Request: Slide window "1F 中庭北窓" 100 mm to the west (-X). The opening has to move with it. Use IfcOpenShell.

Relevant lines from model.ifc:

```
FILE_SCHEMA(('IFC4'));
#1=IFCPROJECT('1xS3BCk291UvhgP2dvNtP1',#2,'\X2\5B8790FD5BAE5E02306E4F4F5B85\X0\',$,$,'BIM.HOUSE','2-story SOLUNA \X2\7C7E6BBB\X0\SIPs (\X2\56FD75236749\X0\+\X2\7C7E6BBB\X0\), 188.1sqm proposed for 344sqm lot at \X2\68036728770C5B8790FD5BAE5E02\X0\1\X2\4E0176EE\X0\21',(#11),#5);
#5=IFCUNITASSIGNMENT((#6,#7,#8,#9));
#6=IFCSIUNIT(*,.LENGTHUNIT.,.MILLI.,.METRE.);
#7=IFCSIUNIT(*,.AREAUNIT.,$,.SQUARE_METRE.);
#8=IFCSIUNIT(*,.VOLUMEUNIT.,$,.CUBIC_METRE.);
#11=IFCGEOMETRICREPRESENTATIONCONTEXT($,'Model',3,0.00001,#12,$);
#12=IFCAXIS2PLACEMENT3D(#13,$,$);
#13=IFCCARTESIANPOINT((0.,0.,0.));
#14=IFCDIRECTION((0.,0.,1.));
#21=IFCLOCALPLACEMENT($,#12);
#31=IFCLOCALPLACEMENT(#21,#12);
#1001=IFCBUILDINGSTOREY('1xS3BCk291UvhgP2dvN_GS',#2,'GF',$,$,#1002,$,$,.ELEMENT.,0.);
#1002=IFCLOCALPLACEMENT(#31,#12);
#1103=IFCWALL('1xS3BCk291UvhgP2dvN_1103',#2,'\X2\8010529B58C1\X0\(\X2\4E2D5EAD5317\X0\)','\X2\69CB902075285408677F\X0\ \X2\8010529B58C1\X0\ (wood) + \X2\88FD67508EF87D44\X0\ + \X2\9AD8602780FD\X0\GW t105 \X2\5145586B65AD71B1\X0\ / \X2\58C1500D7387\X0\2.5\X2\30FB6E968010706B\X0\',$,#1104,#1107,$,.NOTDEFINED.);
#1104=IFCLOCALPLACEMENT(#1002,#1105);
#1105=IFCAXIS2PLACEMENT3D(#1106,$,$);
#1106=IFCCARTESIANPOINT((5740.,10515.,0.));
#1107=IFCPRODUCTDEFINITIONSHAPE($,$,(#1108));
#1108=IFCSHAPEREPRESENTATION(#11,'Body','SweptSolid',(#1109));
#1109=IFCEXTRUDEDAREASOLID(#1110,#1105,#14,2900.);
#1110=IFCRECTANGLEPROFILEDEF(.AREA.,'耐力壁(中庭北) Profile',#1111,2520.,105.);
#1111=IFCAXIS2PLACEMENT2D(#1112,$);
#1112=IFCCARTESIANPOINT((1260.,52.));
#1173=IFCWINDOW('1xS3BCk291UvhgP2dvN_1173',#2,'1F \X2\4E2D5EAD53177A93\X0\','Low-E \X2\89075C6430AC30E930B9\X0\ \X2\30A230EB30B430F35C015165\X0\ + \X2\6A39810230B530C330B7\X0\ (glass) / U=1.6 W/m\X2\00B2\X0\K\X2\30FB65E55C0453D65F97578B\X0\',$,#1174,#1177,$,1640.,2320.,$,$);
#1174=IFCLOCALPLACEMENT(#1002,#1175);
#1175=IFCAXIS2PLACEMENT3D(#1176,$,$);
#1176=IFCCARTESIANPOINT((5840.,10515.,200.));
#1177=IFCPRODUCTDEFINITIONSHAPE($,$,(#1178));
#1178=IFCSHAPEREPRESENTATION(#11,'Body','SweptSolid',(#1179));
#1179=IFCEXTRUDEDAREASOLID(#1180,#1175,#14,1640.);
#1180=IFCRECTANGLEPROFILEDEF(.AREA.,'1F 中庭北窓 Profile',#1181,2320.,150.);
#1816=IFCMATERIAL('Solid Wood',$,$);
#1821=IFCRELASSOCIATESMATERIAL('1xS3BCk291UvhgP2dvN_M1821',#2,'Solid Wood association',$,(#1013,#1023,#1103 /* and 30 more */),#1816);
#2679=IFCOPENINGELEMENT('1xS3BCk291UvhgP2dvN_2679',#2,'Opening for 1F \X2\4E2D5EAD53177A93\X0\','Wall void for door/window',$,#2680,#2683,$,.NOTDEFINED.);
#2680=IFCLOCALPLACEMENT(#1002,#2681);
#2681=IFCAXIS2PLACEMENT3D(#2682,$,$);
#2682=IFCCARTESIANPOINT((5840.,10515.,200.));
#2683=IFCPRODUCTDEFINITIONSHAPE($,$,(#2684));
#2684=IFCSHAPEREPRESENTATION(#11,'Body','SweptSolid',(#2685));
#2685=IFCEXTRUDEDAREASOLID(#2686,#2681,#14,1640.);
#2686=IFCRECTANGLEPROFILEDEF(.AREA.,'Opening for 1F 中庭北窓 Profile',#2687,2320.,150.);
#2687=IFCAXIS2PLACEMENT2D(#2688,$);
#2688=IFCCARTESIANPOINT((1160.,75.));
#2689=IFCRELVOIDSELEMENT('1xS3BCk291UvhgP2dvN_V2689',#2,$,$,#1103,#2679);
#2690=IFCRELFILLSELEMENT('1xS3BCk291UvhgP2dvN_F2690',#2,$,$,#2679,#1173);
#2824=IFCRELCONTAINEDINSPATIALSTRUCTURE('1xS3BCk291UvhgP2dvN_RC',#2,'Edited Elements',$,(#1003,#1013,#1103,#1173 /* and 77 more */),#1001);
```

```python
import ifcopenshell
import ifcopenshell.api.geometry
import ifcopenshell.util.placement
import ifcopenshell.util.unit

model = ifcopenshell.open("model.ifc")
unit_scale = ifcopenshell.util.unit.calculate_unit_scale(model)

window = model.by_id(1173)
opening = window.FillsVoids[0].RelatingOpeningElement
wall = opening.VoidsElements[0].RelatingBuildingElement

wall_matrix = ifcopenshell.util.placement.get_local_placement(wall.ObjectPlacement)
shift = wall_matrix[:3, 0] * -0.1 / unit_scale
before = ifcopenshell.util.placement.get_local_placement(window.ObjectPlacement)[:3, 3].copy()

# The window is not placed relative to its opening, so move both.
for product in (opening, window):
    matrix = ifcopenshell.util.placement.get_local_placement(product.ObjectPlacement)
    matrix[:3, 3] += shift
    ifcopenshell.api.geometry.edit_object_placement(model, product=product, matrix=matrix, is_si=False)

after = ifcopenshell.util.placement.get_local_placement(window.ObjectPlacement)[:3, 3]
print("window moved by", (after - before).round(3) + 0.0)

model.write("model_edited.ifc")
```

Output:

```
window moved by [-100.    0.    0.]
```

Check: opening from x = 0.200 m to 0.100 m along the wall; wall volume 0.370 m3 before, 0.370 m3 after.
